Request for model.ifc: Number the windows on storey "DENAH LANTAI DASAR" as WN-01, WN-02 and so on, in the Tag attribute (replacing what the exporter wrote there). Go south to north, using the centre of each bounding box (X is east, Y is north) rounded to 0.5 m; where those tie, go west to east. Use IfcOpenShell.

First a look at what the model holds.

```python
import ifcopenshell
import ifcopenshell.util.element
import ifcopenshell.util.placement

model = ifcopenshell.open("model.ifc")
print(model.schema)
storey = next(s for s in model.by_type("IfcBuildingStorey") if s.Name == "DENAH LANTAI DASAR")
windows = [e for e in ifcopenshell.util.element.get_decomposition(storey) if e.is_a("IfcWindow")]
for e in sorted(windows, key=lambda e: e.id()):
    origin = ifcopenshell.util.placement.get_local_placement(e.ObjectPlacement)[:3, 3]
    print(e.id(), e.Tag, e.Name, origin.round(2) + 0.0, sep=" | ")
```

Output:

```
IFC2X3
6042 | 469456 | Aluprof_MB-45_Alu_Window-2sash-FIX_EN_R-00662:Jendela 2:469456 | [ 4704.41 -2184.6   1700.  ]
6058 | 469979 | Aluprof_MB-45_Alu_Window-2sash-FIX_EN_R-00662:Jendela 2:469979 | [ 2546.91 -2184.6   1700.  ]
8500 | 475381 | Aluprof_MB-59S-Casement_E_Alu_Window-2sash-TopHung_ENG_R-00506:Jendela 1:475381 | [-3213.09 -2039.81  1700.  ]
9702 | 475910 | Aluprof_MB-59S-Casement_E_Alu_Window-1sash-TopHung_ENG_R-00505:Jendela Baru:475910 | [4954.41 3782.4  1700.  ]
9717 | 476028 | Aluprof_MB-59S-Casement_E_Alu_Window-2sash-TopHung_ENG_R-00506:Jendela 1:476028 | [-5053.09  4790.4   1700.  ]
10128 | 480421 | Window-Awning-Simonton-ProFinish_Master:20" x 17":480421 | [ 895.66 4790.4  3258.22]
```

```python
import ifcopenshell
import ifcopenshell.geom
import ifcopenshell.util.element
import ifcopenshell.util.shape

model = ifcopenshell.open("model.ifc")
settings = ifcopenshell.geom.settings()
settings.set("use-world-coords", True)


def centre(element):
    shape = ifcopenshell.geom.create_shape(settings, element)
    return ifcopenshell.util.shape.get_bbox_centroid(shape.geometry)


storey = next(s for s in model.by_type("IfcBuildingStorey") if s.Name == "DENAH LANTAI DASAR")
windows = [e for e in ifcopenshell.util.element.get_decomposition(storey) if e.is_a("IfcWindow")]

# Insertion points can sit at a corner or the storey origin, so sort by the geometry (in metres).
centres = {e: centre(e) for e in windows}
windows.sort(key=lambda e: (round(centres[e][1] / 0.5), centres[e][0]))

for i, e in enumerate(windows, start=1):
    number = f"WN-{i:02d}"
    e.Tag = number
    print(e.id(), number)

model.write("model_edited.ifc")
```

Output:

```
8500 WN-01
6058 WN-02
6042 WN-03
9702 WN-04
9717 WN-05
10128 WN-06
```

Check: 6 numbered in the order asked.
